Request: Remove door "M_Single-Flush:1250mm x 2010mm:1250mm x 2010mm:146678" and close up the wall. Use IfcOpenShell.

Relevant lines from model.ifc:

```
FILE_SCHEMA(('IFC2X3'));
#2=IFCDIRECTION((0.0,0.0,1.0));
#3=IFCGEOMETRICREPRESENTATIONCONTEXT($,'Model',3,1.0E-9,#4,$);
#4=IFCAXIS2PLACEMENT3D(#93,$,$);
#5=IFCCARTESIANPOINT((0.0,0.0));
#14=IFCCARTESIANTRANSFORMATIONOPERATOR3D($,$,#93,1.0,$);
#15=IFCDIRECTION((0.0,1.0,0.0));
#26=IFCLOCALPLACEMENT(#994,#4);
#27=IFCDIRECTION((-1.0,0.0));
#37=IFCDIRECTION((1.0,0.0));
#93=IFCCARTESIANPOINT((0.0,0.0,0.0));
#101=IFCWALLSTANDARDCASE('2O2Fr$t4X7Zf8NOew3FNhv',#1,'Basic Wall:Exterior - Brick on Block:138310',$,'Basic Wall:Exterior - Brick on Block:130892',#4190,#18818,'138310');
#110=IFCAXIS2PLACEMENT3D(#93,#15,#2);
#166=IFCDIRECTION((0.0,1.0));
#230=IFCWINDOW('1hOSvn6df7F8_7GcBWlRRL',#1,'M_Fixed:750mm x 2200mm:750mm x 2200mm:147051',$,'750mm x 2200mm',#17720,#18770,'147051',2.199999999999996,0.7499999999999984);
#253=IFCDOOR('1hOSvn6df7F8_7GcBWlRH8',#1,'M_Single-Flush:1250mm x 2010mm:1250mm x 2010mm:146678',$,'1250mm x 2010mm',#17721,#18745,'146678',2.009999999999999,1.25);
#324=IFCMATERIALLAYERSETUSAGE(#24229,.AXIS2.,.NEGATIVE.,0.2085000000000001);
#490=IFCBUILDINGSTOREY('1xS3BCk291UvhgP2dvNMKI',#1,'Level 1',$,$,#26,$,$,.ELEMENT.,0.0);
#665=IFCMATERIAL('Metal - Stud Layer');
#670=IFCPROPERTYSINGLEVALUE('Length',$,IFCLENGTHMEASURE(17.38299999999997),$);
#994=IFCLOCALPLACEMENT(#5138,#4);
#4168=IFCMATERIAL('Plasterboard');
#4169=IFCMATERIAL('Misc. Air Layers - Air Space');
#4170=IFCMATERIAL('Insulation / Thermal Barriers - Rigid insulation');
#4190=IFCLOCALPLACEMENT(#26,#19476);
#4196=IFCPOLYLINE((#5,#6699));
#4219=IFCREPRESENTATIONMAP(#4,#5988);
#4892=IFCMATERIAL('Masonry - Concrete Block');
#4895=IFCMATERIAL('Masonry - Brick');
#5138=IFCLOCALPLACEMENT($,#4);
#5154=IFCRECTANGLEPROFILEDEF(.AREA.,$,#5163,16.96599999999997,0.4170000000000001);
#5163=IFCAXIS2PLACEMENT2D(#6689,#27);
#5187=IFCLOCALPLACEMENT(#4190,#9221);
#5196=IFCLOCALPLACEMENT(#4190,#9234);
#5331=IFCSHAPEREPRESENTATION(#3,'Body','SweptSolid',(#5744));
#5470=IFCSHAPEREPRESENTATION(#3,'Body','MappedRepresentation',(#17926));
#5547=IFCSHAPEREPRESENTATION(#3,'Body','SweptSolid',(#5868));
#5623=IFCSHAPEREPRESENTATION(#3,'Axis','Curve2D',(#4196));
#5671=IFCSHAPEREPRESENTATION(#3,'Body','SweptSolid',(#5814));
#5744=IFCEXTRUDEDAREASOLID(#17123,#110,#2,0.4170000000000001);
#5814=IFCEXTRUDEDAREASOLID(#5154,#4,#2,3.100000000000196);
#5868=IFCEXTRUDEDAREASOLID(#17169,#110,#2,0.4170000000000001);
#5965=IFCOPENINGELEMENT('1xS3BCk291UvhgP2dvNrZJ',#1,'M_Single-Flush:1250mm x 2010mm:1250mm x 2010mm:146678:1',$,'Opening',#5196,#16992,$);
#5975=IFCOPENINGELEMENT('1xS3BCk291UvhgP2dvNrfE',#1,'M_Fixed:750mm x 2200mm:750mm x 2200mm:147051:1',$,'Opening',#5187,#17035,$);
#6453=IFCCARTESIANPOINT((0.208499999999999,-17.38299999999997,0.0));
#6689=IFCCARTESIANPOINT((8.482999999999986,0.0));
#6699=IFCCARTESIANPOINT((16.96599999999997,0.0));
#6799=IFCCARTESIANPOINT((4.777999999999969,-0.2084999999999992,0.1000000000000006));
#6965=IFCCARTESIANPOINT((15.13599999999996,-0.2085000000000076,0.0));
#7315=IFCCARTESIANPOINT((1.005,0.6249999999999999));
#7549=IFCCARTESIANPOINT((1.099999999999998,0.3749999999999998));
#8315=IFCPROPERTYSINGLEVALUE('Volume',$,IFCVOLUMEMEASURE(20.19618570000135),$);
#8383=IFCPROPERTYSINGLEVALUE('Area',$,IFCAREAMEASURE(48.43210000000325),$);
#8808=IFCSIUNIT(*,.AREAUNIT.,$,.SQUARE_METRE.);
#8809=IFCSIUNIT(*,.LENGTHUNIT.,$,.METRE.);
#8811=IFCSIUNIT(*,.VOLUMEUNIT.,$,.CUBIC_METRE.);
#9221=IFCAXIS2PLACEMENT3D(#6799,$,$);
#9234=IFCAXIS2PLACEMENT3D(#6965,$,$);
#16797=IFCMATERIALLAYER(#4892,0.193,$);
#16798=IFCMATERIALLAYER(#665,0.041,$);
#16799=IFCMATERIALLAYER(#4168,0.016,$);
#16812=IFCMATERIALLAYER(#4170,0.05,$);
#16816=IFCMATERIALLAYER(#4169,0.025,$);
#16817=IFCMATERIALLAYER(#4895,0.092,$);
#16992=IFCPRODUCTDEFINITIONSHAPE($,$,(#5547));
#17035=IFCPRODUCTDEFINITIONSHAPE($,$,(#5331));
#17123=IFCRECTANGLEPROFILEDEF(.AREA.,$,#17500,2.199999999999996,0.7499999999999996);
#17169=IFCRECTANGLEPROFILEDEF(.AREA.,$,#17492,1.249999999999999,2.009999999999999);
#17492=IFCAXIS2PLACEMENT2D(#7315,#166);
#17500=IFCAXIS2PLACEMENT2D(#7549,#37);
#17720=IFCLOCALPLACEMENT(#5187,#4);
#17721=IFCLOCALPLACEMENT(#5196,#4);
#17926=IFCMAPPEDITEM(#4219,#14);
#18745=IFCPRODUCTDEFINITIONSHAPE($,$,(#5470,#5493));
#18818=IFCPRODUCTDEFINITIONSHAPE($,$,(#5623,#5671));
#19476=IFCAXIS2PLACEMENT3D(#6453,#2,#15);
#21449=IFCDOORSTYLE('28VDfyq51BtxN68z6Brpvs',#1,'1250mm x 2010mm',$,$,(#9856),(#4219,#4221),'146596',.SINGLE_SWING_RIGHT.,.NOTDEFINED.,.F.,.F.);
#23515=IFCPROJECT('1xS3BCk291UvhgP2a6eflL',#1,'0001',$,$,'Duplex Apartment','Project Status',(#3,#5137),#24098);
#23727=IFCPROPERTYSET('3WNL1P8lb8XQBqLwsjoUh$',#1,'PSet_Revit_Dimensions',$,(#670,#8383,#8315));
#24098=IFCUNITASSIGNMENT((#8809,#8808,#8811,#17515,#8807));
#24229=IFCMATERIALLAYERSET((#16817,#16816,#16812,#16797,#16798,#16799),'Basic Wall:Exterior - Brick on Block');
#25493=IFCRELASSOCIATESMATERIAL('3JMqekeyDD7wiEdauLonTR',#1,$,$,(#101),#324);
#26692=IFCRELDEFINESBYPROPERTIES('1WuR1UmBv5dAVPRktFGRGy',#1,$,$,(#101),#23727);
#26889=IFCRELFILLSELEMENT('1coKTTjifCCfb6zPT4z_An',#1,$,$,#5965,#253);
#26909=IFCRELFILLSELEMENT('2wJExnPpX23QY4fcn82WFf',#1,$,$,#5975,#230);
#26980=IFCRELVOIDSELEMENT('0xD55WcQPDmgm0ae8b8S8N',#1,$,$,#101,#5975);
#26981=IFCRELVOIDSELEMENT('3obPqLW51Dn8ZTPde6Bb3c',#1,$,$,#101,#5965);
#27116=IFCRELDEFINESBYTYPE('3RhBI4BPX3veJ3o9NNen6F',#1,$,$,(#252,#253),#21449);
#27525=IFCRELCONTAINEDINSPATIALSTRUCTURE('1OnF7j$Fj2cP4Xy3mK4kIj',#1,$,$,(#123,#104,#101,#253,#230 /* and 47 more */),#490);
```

```python
import ifcopenshell
import ifcopenshell.api.feature
import ifcopenshell.api.pset
import ifcopenshell.api.root
import ifcopenshell.geom
import ifcopenshell.util.element
import ifcopenshell.util.shape
import ifcopenshell.util.unit

model = ifcopenshell.open("model.ifc")
area_scale = ifcopenshell.util.unit.calculate_unit_scale(model, "AREAUNIT")
volume_scale = ifcopenshell.util.unit.calculate_unit_scale(model, "VOLUMEUNIT")
settings = ifcopenshell.geom.settings()


def volume(element):
    """Net volume in cubic metres, openings subtracted."""
    shape = ifcopenshell.geom.create_shape(settings, element)
    return ifcopenshell.util.shape.get_volume(shape.geometry)


door = model.by_guid("1hOSvn6df7F8_7GcBWlRH8")
opening = door.FillsVoids[0].RelatingOpeningElement
wall = opening.VoidsElements[0].RelatingBuildingElement
before = volume(wall)

ifcopenshell.api.root.remove_product(model, product=door)
ifcopenshell.api.feature.remove_feature(model, feature=opening)

after = volume(wall)
thickness = 0.417  # wall thickness in metres

# Update the wall's stored quantities.
pset = model.by_id(ifcopenshell.util.element.get_pset(wall, "PSet_Revit_Dimensions", should_inherit=False)["id"])
ifcopenshell.api.pset.edit_pset(model, pset=pset, properties={
    "Area": model.create_entity("IfcAreaMeasure", after / thickness / area_scale),
    "Volume": model.create_entity("IfcVolumeMeasure", after / volume_scale),
})

print(f"wall volume {before:.3f} -> {after:.3f} m3")

model.write("model-out.ifc")
```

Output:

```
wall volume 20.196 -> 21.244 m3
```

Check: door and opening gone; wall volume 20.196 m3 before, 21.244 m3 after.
